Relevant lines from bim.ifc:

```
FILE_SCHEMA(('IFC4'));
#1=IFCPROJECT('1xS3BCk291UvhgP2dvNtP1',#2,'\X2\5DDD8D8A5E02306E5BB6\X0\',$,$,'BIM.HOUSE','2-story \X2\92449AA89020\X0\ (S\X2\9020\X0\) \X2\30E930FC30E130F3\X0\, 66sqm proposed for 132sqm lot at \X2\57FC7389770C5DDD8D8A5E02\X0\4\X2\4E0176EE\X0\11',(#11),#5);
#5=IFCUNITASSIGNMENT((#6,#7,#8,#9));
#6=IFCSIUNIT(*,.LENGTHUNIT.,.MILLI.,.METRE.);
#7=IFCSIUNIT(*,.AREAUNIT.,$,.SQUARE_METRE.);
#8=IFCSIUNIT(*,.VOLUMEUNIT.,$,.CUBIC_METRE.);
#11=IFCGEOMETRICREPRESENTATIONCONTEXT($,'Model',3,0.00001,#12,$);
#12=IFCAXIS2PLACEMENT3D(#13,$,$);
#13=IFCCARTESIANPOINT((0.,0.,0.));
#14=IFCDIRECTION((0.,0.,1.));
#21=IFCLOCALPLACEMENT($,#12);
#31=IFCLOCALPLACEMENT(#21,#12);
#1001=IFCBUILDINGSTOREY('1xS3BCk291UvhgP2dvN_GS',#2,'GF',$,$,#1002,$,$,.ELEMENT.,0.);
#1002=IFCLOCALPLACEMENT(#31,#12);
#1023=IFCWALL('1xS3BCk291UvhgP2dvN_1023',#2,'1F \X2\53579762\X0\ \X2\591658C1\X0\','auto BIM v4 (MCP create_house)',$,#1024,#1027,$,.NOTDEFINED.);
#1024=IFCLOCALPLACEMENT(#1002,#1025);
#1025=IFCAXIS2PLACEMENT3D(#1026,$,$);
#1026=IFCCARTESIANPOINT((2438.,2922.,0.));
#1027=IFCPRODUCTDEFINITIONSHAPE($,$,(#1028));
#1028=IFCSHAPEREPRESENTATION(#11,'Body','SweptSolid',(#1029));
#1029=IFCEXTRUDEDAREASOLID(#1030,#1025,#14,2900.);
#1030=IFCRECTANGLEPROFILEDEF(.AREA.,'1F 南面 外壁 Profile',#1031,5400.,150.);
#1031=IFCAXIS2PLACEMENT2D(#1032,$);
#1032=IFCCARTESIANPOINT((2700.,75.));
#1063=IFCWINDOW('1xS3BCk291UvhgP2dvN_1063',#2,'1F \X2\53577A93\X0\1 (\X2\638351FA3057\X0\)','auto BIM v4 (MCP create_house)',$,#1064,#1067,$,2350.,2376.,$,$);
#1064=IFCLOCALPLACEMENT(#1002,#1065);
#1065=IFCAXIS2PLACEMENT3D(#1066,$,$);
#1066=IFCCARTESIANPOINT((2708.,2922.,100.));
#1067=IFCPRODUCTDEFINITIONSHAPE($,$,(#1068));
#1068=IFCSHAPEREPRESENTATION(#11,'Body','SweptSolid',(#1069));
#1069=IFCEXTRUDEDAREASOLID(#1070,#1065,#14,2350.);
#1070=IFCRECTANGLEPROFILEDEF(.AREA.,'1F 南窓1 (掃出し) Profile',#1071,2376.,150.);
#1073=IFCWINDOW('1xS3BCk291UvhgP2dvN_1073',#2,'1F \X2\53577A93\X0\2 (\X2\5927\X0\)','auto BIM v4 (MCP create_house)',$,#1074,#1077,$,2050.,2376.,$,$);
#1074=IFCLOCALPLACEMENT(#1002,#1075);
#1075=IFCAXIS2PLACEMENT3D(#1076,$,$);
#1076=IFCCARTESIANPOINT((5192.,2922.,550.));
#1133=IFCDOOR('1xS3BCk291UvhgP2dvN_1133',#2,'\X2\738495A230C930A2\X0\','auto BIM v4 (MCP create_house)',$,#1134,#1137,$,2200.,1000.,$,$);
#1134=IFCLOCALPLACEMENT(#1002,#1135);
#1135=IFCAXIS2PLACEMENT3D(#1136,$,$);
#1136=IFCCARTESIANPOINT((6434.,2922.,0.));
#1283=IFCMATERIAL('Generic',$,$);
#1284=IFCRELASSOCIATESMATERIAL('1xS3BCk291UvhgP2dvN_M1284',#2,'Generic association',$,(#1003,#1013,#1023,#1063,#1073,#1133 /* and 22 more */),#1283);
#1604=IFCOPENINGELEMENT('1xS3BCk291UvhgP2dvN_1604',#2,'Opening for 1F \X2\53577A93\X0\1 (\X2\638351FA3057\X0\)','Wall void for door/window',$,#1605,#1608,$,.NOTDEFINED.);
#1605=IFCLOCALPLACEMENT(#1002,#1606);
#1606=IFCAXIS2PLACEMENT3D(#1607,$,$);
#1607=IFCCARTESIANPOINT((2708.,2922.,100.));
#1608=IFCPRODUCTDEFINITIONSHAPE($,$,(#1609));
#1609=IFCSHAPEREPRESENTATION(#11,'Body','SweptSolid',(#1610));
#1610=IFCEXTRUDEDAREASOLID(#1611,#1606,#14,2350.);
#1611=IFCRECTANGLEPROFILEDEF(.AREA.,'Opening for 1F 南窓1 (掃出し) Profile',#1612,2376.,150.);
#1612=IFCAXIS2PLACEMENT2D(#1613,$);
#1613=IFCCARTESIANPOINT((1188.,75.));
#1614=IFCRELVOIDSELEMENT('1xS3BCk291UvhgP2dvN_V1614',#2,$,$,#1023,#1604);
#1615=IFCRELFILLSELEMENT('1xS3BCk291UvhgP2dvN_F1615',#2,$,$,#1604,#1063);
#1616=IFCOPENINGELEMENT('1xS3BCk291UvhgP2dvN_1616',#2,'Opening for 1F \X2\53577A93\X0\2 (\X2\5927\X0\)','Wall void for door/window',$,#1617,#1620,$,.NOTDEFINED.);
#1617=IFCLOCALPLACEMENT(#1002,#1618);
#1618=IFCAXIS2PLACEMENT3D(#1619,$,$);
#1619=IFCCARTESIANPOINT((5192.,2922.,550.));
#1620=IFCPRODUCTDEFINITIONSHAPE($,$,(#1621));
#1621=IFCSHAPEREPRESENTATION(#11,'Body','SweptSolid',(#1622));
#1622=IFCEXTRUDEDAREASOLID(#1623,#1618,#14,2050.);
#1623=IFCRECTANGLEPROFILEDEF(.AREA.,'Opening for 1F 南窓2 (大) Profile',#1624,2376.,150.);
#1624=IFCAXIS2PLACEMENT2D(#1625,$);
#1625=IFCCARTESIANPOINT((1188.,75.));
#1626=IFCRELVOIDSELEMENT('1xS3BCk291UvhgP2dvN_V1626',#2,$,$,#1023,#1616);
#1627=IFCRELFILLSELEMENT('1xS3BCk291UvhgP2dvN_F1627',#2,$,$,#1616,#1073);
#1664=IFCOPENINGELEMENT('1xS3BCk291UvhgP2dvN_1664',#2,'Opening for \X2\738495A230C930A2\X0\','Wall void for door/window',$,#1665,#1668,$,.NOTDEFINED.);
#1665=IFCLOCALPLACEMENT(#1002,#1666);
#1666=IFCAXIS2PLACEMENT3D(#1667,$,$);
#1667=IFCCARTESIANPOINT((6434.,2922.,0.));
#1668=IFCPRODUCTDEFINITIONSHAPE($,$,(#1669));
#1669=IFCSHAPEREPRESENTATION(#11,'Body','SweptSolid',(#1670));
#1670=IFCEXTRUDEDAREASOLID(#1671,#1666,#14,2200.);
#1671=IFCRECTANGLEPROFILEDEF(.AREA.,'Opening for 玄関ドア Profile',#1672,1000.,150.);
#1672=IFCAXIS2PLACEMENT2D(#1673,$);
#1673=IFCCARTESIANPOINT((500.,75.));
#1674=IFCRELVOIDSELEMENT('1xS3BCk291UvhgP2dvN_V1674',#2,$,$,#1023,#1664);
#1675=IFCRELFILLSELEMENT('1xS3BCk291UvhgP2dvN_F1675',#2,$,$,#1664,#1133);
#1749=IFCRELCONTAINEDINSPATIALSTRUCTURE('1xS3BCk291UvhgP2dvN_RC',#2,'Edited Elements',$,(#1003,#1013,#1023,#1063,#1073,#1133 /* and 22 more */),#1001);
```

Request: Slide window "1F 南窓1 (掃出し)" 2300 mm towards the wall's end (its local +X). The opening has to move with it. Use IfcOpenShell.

```python
import ifcopenshell
import ifcopenshell.api.geometry
import ifcopenshell.util.placement
import ifcopenshell.util.unit

model = ifcopenshell.open("bim.ifc")
unit_scale = ifcopenshell.util.unit.calculate_unit_scale(model)

window = model.by_guid("1xS3BCk291UvhgP2dvN_1063")
opening = window.FillsVoids[0].RelatingOpeningElement
wall = opening.VoidsElements[0].RelatingBuildingElement

wall_matrix = ifcopenshell.util.placement.get_local_placement(wall.ObjectPlacement)
shift = wall_matrix[:3, 0] * 2.3 / unit_scale
before = ifcopenshell.util.placement.get_local_placement(window.ObjectPlacement)[:3, 3].copy()

# The window is not placed relative to its opening, so move both.
for product in (opening, window):
    matrix = ifcopenshell.util.placement.get_local_placement(product.ObjectPlacement)
    matrix[:3, 3] += shift
    ifcopenshell.api.geometry.edit_object_placement(model, product=product, matrix=matrix, is_si=False)

after = ifcopenshell.util.placement.get_local_placement(window.ObjectPlacement)[:3, 3]
print("window moved by", (after - before).round(3) + 0.0)

model.write("bim_rev.ifc")
```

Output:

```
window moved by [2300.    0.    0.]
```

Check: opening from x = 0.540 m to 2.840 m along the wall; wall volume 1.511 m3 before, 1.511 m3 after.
